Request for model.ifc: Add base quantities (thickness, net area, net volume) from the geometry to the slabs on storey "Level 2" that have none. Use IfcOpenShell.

First a look at what the model holds.

```python
import ifcopenshell
import ifcopenshell.util.element
import ifcopenshell.util.unit

model = ifcopenshell.open("model.ifc")
print(model.schema)
for unit_type in ("LENGTHUNIT", "AREAUNIT", "VOLUMEUNIT"):
    print(unit_type, ifcopenshell.util.unit.calculate_unit_scale(model, unit_type))
storey = next(s for s in model.by_type("IfcBuildingStorey") if s.Name == "Level 2")
slabs = [e for e in ifcopenshell.util.element.get_decomposition(storey) if e.is_a("IfcSlab")]
for e in sorted(slabs, key=lambda e: e.id()):
    print(e.id(), e.is_a(), e.Name, list(ifcopenshell.util.element.get_psets(e, qtos_only=True)), sep=" | ")
```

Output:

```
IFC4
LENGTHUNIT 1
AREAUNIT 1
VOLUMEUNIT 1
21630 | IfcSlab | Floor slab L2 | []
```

```python
import ifcopenshell
import ifcopenshell.api.pset
import ifcopenshell.geom
import ifcopenshell.util.element
import ifcopenshell.util.shape
import ifcopenshell.util.unit

model = ifcopenshell.open("model.ifc")
unit_scale = ifcopenshell.util.unit.calculate_unit_scale(model)
area_scale = ifcopenshell.util.unit.calculate_unit_scale(model, "AREAUNIT")
volume_scale = ifcopenshell.util.unit.calculate_unit_scale(model, "VOLUMEUNIT")
settings = ifcopenshell.geom.settings()

storey = next(s for s in model.by_type("IfcBuildingStorey") if s.Name == "Level 2")
slabs = [e for e in ifcopenshell.util.element.get_decomposition(storey) if e.is_a("IfcSlab")]

for e in sorted(slabs, key=lambda e: e.id()):
    if ifcopenshell.util.element.get_psets(e, qtos_only=True, should_inherit=False):
        continue
    # Geometry comes back in metres, in the element's own axes.
    shape = ifcopenshell.geom.create_shape(settings, e)
    values = {
        "Width": ifcopenshell.util.shape.get_z(shape.geometry) / unit_scale,
        "NetArea": ifcopenshell.util.shape.get_footprint_area(shape.geometry) / area_scale,
        "NetVolume": ifcopenshell.util.shape.get_volume(shape.geometry) / volume_scale,
    }
    qto = ifcopenshell.api.pset.add_qto(model, product=e, name="Qto_SlabBaseQuantities")
    ifcopenshell.api.pset.edit_qto(model, qto=qto, properties=values)
    print(e.id(), {k: round(v, 3) for k, v in values.items()})

model.write("model_rev.ifc")
```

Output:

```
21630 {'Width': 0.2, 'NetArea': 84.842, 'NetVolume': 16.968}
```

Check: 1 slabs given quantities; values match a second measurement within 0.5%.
